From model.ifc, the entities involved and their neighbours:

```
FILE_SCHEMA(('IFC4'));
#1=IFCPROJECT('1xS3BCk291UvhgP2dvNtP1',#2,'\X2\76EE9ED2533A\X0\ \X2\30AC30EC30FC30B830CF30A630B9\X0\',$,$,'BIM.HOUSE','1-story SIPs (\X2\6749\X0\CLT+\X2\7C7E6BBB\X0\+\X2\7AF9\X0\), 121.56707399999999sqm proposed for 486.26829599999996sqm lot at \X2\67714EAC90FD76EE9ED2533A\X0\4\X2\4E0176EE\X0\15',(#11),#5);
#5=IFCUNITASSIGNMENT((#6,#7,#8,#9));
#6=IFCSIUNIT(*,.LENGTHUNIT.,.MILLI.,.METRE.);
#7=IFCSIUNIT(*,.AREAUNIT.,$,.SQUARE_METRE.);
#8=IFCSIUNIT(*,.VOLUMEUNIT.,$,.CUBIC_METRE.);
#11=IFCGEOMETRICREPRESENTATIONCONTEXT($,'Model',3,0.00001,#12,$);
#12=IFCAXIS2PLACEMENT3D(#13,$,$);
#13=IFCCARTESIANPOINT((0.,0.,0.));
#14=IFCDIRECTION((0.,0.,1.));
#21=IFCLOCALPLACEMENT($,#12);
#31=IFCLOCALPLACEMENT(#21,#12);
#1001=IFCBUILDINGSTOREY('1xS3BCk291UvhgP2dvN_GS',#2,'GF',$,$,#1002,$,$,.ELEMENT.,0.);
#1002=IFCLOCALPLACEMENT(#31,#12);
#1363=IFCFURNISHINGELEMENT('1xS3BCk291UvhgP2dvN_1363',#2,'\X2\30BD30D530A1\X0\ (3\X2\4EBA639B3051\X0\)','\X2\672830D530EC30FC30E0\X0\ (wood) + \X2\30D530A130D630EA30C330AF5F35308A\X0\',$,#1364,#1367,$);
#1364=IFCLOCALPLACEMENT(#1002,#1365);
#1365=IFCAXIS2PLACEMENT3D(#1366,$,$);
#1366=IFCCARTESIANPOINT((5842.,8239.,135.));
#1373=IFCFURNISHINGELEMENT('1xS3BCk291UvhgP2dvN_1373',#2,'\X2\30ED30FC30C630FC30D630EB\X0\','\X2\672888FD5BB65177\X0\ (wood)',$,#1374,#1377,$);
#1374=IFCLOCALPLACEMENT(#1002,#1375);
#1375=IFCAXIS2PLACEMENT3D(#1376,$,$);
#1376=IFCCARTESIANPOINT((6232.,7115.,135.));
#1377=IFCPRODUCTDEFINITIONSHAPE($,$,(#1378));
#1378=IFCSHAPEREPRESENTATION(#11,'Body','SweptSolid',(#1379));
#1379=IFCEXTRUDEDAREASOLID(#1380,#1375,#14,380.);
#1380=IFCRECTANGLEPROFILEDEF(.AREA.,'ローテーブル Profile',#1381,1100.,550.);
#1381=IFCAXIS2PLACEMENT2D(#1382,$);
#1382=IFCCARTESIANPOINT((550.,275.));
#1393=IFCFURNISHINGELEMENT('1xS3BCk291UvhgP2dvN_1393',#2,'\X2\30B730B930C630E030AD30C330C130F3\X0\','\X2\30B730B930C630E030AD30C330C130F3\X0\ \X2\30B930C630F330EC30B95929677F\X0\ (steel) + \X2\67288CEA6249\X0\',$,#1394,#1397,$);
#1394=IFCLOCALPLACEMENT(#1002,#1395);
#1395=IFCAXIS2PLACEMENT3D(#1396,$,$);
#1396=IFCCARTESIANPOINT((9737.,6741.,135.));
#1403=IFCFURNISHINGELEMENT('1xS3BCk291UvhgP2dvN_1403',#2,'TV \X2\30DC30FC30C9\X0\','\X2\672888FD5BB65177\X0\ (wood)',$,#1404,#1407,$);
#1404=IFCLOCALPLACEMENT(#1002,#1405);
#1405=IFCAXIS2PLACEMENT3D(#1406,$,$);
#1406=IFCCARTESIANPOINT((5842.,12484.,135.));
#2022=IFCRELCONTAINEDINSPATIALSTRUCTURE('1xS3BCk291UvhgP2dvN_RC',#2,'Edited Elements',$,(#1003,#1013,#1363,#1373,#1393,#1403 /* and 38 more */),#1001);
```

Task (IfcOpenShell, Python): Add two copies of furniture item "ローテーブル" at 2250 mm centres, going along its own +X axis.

```python
import ifcopenshell
import ifcopenshell.api.geometry
import ifcopenshell.api.root
import ifcopenshell.util.element
import ifcopenshell.util.placement
import ifcopenshell.util.unit

model = ifcopenshell.open("model.ifc")
unit_scale = ifcopenshell.util.unit.calculate_unit_scale(model)


def reuse_history(source, copy):
    """copy_class also copies each property set's owner history, people and application; keep the originals."""
    for rel in copy.IsDefinedBy:
        if rel.is_a("IfcRelDefinesByProperties") and (history := rel.RelatingPropertyDefinition.OwnerHistory):
            rel.RelatingPropertyDefinition.OwnerHistory = source.OwnerHistory
            ifcopenshell.util.element.remove_deep2(model, history)


source = model.by_id(1373)
base = ifcopenshell.util.placement.get_local_placement(source.ObjectPlacement)
step = base[:3, 0] * 2.25 / unit_scale

for i in range(1, 3):
    copy = ifcopenshell.api.root.copy_class(model, product=source)
    copy.Representation = ifcopenshell.util.element.copy_deep(
        model, source.Representation, exclude=["IfcGeometricRepresentationContext", "IfcRepresentationMap"]
    )
    reuse_history(source, copy)
    matrix = base.copy()
    matrix[:3, 3] += i * step
    print("added at", matrix[:3, 3].round(3) + 0.0)
    ifcopenshell.api.geometry.edit_object_placement(model, product=copy, matrix=matrix, is_si=False)

model.write("model_rev.ifc")
```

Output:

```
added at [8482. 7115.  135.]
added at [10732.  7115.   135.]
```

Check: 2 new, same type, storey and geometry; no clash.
